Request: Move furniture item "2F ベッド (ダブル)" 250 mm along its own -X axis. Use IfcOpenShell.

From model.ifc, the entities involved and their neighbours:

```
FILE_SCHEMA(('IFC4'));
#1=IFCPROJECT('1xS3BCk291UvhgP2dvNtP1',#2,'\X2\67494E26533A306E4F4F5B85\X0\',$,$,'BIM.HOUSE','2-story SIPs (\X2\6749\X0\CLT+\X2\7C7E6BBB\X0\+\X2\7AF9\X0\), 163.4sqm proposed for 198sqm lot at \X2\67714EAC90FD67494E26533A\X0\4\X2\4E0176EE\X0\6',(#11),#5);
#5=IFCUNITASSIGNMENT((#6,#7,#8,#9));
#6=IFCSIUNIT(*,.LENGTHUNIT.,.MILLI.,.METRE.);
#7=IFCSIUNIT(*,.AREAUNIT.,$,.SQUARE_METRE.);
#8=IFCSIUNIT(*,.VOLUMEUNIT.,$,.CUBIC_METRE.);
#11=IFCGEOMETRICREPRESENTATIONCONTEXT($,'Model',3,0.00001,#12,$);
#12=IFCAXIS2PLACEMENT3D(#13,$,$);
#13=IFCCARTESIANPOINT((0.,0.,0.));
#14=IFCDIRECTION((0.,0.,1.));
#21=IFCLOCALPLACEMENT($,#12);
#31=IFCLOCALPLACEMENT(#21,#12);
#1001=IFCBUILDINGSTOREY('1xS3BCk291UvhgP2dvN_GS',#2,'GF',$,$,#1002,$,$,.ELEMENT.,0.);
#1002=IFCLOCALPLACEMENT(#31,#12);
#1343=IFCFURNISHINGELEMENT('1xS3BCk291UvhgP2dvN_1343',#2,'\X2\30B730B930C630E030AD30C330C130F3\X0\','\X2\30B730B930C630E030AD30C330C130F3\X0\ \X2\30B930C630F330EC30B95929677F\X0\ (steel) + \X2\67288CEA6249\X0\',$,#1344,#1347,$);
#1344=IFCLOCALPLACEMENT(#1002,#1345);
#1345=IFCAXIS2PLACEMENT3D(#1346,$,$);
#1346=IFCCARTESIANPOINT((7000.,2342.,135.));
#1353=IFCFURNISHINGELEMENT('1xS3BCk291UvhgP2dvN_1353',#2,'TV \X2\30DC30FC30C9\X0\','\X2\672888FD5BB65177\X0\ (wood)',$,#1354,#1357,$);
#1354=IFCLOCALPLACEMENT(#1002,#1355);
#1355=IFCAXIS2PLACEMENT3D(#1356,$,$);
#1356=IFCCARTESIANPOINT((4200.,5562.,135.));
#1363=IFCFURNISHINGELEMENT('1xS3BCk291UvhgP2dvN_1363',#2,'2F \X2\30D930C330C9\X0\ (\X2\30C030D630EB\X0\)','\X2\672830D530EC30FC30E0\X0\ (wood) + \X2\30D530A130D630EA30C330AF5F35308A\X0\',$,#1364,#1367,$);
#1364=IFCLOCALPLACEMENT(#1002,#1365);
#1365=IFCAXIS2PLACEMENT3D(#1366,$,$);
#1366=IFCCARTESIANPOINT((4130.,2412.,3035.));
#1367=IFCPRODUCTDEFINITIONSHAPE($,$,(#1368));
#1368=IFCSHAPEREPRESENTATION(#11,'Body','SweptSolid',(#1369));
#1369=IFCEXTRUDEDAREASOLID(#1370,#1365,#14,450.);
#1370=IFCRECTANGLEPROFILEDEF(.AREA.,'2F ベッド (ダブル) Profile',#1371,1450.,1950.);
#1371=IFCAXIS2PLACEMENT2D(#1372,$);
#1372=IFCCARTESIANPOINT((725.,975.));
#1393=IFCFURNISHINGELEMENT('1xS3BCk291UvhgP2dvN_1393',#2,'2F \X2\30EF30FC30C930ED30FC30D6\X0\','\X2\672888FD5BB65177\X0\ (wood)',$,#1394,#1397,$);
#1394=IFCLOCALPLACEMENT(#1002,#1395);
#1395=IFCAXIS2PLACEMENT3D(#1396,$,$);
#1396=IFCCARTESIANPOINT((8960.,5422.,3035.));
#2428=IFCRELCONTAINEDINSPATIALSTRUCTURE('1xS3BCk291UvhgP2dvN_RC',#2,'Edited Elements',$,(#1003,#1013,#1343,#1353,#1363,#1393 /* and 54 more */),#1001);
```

```python
import ifcopenshell
import ifcopenshell.api.geometry
import ifcopenshell.util.placement

model = ifcopenshell.open("model.ifc")

item = model.by_guid("1xS3BCk291UvhgP2dvN_1363")
matrix = ifcopenshell.util.placement.get_local_placement(item.ObjectPlacement)
matrix[:3, 3] -= matrix[:3, 0] * 250.0
ifcopenshell.api.geometry.edit_object_placement(model, product=item, matrix=matrix, is_si=False)

print(ifcopenshell.util.placement.get_local_placement(item.ObjectPlacement).round(3) + 0.0)

model.write("model_rev.ifc")
```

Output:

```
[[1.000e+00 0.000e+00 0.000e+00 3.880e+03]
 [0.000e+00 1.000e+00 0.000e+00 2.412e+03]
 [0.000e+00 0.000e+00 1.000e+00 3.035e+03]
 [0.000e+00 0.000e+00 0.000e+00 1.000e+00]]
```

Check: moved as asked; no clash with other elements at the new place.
